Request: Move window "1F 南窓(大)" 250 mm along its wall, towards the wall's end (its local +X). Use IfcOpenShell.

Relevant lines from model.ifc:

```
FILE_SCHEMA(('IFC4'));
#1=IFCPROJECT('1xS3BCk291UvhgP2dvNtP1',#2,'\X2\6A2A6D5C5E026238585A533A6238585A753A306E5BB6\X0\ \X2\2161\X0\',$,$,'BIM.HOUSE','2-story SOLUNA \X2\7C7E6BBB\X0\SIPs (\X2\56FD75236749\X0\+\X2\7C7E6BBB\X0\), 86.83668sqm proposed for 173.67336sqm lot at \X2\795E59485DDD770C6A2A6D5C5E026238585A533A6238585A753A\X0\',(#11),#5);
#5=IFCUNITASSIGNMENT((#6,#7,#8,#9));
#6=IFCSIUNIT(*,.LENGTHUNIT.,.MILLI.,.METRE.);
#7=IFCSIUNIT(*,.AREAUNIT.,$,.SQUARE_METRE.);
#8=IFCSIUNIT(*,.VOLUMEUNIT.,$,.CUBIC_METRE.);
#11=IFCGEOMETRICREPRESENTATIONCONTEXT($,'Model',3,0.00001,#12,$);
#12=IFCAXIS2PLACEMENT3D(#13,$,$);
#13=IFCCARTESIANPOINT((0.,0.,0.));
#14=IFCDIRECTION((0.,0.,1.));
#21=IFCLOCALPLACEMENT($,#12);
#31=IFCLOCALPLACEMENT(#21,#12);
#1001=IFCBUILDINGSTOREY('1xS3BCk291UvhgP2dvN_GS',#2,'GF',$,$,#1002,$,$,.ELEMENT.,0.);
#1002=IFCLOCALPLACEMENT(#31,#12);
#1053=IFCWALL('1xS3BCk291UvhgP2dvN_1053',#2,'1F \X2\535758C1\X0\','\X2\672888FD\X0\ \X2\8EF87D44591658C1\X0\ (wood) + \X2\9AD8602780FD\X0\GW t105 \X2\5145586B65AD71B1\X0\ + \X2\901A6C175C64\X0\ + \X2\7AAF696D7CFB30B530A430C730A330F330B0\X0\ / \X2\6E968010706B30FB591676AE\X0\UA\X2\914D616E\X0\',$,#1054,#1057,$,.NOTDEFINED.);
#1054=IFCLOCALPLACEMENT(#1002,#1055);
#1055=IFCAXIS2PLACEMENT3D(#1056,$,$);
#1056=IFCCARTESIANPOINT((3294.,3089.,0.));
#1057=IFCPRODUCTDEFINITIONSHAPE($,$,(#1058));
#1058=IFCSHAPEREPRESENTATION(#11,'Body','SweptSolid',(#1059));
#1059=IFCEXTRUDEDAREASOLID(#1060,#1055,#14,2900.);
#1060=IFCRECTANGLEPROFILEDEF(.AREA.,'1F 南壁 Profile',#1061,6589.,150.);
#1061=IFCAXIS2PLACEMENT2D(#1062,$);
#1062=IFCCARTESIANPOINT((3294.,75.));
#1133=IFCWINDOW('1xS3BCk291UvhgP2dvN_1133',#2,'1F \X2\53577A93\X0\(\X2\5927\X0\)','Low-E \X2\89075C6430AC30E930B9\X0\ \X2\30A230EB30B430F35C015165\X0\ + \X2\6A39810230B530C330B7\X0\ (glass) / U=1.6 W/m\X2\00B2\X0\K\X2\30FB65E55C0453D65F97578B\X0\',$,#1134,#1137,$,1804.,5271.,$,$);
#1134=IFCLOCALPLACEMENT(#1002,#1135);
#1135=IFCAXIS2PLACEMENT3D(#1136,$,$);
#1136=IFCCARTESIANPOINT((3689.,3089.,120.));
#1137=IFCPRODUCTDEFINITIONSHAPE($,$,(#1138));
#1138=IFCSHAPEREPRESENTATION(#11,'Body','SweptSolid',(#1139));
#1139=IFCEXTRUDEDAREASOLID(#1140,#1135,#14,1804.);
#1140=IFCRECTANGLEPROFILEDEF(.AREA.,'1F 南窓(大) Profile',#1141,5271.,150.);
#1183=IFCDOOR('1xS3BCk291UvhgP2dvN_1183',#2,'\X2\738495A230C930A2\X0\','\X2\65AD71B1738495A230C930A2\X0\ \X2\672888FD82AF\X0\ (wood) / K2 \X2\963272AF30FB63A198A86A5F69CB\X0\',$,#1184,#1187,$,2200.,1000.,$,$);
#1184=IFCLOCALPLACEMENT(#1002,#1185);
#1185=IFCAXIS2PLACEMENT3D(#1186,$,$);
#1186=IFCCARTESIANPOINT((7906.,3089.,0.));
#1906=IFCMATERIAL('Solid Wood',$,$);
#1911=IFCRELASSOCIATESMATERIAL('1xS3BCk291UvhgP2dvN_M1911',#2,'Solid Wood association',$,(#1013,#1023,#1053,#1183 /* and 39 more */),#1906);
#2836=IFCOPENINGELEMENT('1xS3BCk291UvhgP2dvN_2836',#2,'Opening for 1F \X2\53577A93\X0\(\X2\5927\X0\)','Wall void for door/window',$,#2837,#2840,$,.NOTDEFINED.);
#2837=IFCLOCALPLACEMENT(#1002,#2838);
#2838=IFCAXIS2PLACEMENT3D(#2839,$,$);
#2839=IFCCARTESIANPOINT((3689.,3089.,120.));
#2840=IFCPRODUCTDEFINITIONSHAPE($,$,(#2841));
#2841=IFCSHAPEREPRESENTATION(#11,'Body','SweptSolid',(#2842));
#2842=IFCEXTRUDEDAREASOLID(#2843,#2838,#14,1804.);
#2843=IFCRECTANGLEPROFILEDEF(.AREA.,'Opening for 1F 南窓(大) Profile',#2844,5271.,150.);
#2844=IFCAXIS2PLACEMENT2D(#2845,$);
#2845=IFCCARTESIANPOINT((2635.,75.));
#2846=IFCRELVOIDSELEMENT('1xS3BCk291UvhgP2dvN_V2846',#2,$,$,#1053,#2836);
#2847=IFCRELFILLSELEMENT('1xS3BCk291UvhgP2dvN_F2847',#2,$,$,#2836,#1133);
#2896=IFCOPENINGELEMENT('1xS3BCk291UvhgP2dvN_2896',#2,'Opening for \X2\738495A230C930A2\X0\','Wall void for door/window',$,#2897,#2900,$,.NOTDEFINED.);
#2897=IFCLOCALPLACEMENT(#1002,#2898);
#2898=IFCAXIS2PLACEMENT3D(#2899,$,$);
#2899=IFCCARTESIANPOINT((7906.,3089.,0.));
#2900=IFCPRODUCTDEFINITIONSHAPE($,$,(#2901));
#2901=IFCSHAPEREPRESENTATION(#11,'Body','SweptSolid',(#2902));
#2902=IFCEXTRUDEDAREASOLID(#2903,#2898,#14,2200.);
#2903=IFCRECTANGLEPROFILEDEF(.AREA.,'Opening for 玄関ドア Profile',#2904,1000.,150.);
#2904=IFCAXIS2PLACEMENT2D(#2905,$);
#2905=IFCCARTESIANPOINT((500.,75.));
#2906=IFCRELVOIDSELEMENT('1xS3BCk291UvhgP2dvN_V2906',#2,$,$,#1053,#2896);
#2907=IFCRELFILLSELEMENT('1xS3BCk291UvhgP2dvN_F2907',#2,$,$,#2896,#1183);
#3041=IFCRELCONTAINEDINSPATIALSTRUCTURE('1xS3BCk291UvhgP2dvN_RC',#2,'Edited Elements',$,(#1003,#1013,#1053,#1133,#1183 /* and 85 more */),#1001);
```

```python
import ifcopenshell
import ifcopenshell.api.geometry
import ifcopenshell.util.placement

model = ifcopenshell.open("model.ifc")

window = model.by_guid("1xS3BCk291UvhgP2dvN_1133")
opening = window.FillsVoids[0].RelatingOpeningElement
wall = opening.VoidsElements[0].RelatingBuildingElement

wall_matrix = ifcopenshell.util.placement.get_local_placement(wall.ObjectPlacement)
shift = wall_matrix[:3, 0] * 250.0
before = ifcopenshell.util.placement.get_local_placement(window.ObjectPlacement)[:3, 3].copy()

# The window is not placed relative to its opening, so move both.
for product in (opening, window):
    matrix = ifcopenshell.util.placement.get_local_placement(product.ObjectPlacement)
    matrix[:3, 3] += shift
    ifcopenshell.api.geometry.edit_object_placement(model, product=product, matrix=matrix, is_si=False)

after = ifcopenshell.util.placement.get_local_placement(window.ObjectPlacement)[:3, 3]
print("window moved by", (after - before).round(3) + 0.0)

model.write("model_updated.ifc")
```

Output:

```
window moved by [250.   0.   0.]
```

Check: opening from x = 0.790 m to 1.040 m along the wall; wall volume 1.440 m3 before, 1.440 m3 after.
